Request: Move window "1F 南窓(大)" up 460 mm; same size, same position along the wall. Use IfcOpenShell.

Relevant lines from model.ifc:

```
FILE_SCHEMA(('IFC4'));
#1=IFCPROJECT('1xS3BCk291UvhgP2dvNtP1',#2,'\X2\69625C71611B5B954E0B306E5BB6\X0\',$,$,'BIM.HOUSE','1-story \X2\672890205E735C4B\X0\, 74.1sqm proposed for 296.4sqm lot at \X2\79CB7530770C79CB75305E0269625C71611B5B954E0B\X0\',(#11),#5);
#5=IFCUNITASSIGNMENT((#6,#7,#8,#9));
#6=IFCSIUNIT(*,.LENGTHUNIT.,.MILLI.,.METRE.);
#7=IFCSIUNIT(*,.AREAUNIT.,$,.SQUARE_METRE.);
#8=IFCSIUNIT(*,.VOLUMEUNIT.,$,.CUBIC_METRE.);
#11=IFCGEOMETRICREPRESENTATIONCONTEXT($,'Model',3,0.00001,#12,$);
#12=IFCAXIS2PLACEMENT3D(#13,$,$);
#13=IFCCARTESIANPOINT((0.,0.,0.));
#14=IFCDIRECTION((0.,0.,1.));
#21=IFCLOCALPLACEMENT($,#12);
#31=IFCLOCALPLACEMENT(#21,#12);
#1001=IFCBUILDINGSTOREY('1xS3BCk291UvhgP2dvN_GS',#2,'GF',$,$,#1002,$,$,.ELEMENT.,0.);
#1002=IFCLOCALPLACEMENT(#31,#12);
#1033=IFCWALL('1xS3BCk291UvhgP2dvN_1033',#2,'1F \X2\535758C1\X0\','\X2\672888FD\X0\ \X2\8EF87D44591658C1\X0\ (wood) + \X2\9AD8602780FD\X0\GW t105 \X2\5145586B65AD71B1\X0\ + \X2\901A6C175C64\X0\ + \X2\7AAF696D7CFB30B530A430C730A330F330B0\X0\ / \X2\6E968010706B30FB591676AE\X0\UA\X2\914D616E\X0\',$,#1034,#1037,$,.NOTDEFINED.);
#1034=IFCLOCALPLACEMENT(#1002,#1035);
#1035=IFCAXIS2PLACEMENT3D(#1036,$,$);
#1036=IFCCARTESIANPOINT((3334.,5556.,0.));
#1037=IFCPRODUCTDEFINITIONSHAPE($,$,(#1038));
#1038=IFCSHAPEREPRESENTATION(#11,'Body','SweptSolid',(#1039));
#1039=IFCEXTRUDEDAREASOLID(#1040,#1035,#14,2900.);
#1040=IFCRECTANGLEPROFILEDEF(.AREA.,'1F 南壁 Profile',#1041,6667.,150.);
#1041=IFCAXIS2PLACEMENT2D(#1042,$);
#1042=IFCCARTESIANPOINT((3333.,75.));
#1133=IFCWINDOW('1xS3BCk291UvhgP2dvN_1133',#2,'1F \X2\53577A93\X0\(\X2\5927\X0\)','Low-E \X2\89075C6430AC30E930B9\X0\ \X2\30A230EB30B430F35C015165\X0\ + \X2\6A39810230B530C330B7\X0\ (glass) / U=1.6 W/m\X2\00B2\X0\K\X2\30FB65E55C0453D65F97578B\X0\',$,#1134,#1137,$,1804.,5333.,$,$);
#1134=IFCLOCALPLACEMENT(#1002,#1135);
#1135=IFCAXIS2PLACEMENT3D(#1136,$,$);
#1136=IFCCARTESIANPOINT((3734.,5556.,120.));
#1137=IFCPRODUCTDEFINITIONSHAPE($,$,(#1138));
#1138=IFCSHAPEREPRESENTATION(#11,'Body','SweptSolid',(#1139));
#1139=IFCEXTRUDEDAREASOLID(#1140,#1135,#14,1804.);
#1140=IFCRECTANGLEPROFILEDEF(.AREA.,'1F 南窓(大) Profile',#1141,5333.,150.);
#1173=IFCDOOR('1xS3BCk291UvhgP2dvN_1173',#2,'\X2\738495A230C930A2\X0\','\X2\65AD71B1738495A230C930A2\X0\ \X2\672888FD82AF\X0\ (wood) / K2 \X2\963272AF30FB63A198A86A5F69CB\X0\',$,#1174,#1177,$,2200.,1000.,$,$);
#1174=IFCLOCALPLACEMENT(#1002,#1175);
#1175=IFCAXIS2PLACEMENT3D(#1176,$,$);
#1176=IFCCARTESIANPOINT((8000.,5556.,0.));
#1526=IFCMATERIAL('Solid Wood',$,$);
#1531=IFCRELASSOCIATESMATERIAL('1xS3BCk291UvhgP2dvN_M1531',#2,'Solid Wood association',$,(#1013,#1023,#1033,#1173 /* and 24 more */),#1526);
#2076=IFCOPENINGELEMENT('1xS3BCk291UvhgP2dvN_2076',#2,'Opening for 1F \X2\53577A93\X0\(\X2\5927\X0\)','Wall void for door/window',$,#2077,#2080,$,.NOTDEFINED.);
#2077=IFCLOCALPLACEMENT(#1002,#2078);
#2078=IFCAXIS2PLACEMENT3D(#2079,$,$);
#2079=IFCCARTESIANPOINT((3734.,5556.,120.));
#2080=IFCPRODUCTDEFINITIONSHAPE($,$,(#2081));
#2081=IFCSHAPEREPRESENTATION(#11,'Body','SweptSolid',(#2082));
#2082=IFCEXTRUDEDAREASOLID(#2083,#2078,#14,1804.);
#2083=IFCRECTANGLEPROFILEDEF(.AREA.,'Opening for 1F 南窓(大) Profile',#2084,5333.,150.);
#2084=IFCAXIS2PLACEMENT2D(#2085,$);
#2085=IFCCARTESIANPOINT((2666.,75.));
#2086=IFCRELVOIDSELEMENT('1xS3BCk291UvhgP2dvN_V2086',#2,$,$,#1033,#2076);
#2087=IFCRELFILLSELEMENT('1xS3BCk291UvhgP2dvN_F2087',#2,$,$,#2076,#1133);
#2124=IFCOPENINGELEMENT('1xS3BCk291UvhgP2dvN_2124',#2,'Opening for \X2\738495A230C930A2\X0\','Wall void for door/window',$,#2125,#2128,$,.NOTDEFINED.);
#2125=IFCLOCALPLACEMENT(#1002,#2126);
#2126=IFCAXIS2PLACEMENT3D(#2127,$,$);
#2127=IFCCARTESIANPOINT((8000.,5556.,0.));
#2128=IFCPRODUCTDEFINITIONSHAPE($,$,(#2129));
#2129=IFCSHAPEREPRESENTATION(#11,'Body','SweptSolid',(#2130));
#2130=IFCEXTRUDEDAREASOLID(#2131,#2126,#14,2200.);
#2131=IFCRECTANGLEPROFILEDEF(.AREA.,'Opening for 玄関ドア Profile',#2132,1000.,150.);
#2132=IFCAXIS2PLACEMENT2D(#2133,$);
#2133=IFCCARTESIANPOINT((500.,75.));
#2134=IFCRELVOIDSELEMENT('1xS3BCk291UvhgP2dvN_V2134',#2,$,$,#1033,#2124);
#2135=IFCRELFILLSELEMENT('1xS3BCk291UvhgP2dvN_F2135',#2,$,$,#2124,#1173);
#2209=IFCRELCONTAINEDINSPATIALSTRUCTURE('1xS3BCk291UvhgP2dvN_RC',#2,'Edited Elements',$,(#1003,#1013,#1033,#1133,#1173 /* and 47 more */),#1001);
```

```python
import numpy as np
import ifcopenshell
import ifcopenshell.api.geometry
import ifcopenshell.util.placement
import ifcopenshell.util.unit

model = ifcopenshell.open("model.ifc")
unit_scale = ifcopenshell.util.unit.calculate_unit_scale(model)

window = model.by_guid("1xS3BCk291UvhgP2dvN_1133")
opening = window.FillsVoids[0].RelatingOpeningElement
dz = 0.46 / unit_scale

shift = np.array([0.0, 0.0, dz])
# The window is not placed relative to its opening, so move both.
for product in (opening, window):
    matrix = ifcopenshell.util.placement.get_local_placement(product.ObjectPlacement)
    matrix[:3, 3] += shift
    ifcopenshell.api.geometry.edit_object_placement(model, product=product, matrix=matrix, is_si=False)

print(f"moved by {dz * unit_scale:+.3f} m")

model.write("model_updated.ifc")
```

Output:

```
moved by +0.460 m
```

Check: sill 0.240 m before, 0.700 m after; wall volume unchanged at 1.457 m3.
